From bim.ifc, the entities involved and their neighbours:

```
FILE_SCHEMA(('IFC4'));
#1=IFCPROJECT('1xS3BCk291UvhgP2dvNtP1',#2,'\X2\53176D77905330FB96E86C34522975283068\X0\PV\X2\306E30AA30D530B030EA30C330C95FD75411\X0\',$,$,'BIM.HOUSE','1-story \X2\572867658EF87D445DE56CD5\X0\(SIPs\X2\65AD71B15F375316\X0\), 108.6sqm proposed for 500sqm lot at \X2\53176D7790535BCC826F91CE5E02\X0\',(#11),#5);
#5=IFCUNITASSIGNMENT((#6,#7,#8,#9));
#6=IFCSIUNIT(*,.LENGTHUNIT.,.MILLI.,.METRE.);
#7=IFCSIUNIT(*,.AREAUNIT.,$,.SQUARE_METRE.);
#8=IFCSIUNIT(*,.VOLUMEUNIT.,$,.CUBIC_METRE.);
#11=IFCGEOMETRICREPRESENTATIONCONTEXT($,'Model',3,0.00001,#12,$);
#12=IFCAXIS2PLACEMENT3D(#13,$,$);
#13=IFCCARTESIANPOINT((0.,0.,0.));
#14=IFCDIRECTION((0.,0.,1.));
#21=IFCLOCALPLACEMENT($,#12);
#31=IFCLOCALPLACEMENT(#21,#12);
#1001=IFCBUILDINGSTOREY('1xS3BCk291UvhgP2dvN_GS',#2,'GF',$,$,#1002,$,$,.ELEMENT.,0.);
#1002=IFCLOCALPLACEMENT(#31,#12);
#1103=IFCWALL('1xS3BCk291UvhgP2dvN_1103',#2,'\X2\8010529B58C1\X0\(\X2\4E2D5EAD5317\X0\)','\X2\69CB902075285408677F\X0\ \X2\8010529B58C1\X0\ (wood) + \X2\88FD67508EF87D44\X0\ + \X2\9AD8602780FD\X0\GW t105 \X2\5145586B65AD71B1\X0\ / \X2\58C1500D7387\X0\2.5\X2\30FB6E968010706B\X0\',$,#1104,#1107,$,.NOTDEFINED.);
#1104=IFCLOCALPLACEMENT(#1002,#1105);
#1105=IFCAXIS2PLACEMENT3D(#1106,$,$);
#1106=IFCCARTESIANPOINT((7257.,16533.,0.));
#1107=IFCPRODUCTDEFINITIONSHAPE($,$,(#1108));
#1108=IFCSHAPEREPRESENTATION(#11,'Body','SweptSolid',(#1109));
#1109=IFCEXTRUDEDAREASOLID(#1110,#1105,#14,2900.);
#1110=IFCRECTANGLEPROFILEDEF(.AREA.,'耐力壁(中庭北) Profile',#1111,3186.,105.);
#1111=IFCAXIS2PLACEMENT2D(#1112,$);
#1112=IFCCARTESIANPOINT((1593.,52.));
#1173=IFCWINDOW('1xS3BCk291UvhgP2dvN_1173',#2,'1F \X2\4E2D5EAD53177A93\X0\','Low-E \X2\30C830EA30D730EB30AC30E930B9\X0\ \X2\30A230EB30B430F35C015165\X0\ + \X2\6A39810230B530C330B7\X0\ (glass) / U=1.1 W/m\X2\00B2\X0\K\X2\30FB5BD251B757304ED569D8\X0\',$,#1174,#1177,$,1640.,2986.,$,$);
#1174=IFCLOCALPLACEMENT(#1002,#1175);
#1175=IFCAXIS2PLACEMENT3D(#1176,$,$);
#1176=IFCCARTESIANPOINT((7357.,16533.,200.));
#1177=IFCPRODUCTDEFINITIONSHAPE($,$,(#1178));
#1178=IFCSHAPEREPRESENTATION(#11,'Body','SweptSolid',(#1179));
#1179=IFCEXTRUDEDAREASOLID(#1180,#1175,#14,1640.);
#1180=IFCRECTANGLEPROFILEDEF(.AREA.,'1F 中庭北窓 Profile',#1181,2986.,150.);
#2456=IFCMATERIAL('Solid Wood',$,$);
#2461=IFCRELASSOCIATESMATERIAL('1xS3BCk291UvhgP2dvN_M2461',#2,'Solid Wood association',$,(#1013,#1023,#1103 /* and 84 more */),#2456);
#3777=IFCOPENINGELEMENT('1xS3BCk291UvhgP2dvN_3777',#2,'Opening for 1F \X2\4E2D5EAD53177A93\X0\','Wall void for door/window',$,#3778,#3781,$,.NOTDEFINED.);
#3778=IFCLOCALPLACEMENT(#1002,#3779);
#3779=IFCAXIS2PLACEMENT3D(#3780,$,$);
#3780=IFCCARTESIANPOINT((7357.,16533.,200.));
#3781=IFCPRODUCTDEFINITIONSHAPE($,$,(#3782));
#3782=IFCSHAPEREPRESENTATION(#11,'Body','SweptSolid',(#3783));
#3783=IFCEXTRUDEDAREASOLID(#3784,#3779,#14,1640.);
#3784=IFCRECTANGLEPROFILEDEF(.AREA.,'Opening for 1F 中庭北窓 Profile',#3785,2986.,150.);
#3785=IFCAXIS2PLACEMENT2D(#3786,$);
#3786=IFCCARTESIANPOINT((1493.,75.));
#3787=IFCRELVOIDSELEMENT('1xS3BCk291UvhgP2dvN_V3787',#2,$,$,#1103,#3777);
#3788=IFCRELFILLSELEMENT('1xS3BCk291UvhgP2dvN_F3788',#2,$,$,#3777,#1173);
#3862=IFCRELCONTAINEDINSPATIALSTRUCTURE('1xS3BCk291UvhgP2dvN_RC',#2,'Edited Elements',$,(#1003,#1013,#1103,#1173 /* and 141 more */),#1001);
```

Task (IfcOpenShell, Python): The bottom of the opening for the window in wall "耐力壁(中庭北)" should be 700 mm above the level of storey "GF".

```python
import numpy as np
import ifcopenshell
import ifcopenshell.api.geometry
import ifcopenshell.geom
import ifcopenshell.util.element
import ifcopenshell.util.placement
import ifcopenshell.util.shape
import ifcopenshell.util.unit

model = ifcopenshell.open("bim.ifc")
unit_scale = ifcopenshell.util.unit.calculate_unit_scale(model)

window = model.by_guid("1xS3BCk291UvhgP2dvN_1173")
opening = window.FillsVoids[0].RelatingOpeningElement
storey = ifcopenshell.util.element.get_container(window, ifc_class="IfcBuildingStorey")
level = ifcopenshell.util.placement.get_local_placement(storey.ObjectPlacement)[2, 3]

# The opening's origin need not be at the sill, so measure its lowest point.
shape = ifcopenshell.geom.create_shape(ifcopenshell.geom.settings(), opening)
bottom = ifcopenshell.util.shape.get_shape_bottom_elevation(shape, shape.geometry) / unit_scale
dz = level + 700.0 - bottom

shift = np.array([0.0, 0.0, dz])
# The window is not placed relative to its opening, so move both.
for product in (opening, window):
    matrix = ifcopenshell.util.placement.get_local_placement(product.ObjectPlacement)
    matrix[:3, 3] += shift
    ifcopenshell.api.geometry.edit_object_placement(model, product=product, matrix=matrix, is_si=False)

print(f"moved by {dz * unit_scale:+.3f} m")

model.write("bim_updated.ifc")
```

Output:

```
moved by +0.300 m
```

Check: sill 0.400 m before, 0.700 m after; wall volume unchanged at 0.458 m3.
